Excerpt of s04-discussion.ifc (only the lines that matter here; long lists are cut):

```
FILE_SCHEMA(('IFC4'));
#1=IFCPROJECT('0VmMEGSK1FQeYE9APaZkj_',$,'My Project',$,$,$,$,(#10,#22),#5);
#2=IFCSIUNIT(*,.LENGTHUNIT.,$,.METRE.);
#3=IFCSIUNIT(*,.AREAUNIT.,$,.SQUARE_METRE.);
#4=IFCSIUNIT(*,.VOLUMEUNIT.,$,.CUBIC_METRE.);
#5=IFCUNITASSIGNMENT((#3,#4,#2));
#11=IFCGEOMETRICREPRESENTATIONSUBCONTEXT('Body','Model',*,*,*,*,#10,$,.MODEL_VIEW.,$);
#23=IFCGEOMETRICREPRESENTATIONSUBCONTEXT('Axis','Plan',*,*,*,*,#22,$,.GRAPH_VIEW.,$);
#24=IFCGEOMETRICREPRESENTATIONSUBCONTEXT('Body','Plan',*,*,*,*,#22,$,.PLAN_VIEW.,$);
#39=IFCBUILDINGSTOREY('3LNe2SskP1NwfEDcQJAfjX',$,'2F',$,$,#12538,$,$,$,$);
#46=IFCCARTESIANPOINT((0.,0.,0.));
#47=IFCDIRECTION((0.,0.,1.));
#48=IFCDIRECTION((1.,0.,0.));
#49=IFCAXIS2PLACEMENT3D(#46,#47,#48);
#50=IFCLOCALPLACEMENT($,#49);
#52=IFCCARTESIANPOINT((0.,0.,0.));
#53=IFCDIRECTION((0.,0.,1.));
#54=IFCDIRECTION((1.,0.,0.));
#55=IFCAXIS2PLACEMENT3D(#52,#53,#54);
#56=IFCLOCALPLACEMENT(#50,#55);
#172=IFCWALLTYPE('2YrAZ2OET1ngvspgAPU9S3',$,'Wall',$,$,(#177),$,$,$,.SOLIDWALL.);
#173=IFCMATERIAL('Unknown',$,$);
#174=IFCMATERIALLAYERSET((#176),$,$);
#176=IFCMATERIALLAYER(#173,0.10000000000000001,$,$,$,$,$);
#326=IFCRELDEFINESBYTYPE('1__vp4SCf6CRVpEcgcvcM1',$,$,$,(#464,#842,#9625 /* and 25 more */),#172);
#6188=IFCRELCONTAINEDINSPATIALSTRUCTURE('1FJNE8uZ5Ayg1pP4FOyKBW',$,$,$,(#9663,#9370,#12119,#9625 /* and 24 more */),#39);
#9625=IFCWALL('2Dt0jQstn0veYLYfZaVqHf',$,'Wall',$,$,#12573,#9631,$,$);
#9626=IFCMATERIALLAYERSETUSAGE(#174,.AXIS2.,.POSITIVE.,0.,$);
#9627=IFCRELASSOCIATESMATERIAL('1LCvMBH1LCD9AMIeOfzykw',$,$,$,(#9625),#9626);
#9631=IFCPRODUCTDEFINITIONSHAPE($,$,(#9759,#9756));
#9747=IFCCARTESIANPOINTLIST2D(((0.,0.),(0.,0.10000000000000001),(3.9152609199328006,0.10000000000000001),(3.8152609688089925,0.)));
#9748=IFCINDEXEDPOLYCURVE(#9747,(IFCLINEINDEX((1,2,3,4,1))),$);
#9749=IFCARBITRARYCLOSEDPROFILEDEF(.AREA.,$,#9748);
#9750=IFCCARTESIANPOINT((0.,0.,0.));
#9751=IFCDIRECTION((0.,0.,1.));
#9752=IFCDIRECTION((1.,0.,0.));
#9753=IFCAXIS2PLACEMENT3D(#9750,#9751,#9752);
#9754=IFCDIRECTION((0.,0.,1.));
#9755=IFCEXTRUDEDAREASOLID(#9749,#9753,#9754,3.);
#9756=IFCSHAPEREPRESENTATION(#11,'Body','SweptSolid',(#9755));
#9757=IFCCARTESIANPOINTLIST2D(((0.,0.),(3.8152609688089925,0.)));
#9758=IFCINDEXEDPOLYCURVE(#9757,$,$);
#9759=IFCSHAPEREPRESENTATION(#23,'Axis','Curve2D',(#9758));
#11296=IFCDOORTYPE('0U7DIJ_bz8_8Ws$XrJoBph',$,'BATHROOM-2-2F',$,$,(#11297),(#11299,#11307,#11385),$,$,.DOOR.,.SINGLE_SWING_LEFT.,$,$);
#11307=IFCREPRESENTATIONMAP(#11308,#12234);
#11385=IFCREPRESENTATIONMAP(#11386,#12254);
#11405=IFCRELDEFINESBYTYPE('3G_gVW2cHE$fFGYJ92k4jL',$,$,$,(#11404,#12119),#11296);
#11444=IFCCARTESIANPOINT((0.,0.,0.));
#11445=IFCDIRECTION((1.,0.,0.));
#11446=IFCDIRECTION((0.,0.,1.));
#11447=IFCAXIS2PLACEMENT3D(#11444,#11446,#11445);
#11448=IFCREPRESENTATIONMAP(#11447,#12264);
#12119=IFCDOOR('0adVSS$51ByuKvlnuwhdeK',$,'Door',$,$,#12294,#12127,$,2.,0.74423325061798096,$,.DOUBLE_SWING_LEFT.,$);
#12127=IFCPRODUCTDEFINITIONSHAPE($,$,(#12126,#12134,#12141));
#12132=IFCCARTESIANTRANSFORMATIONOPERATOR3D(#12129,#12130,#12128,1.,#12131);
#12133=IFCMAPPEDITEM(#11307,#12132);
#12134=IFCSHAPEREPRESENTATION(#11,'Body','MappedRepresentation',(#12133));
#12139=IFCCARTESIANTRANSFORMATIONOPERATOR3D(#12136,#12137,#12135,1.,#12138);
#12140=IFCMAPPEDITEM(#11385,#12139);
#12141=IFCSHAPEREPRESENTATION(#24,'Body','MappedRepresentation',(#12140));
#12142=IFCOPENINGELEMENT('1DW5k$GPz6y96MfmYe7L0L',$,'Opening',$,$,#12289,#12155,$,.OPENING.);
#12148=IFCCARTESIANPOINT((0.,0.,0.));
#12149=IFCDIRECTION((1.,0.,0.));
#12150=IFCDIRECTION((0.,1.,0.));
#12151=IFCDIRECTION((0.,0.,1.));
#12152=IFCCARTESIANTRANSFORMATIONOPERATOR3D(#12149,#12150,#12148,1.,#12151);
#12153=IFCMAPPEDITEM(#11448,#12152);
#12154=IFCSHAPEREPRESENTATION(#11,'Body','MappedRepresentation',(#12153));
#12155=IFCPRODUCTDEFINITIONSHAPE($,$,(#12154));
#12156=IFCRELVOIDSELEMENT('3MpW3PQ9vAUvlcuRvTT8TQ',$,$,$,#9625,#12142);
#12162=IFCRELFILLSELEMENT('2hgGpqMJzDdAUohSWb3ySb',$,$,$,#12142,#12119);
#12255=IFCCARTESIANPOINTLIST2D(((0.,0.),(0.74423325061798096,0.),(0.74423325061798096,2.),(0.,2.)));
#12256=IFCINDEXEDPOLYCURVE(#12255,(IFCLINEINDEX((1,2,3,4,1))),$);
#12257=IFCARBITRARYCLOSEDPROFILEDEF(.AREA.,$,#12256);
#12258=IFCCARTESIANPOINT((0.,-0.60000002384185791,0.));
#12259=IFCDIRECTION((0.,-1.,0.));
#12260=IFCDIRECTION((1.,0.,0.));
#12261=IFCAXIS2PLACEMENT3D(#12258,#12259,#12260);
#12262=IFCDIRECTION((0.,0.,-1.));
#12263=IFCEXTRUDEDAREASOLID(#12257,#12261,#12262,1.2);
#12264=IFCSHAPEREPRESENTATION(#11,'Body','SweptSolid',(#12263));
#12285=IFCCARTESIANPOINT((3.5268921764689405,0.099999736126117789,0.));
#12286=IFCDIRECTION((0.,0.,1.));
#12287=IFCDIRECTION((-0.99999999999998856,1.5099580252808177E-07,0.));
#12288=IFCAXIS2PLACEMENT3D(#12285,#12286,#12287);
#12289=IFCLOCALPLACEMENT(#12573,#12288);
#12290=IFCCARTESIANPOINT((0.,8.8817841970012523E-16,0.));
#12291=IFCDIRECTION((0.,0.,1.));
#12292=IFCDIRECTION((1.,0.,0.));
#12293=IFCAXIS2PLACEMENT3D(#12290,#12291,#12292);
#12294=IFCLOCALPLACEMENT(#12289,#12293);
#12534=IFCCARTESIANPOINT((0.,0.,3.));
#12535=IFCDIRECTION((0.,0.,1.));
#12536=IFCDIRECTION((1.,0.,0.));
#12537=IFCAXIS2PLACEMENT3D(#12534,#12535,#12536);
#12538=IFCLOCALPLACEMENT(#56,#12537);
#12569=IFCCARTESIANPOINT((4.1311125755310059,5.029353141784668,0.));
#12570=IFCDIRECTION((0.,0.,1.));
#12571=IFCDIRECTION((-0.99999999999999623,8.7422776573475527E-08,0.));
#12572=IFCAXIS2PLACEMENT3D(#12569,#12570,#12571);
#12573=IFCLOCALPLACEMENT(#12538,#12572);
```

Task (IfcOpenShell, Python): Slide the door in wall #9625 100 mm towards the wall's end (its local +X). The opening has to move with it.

```python
import ifcopenshell
import ifcopenshell.api.geometry
import ifcopenshell.util.placement

model = ifcopenshell.open("s04-discussion.ifc")

door = model.by_guid("0adVSS$51ByuKvlnuwhdeK")
opening = door.FillsVoids[0].RelatingOpeningElement
wall = opening.VoidsElements[0].RelatingBuildingElement

wall_matrix = ifcopenshell.util.placement.get_local_placement(wall.ObjectPlacement)
shift = wall_matrix[:3, 0] * 0.1
before = ifcopenshell.util.placement.get_local_placement(door.ObjectPlacement)[:3, 3].copy()

# The door is placed relative to its opening, so it follows when the opening moves.
matrix = ifcopenshell.util.placement.get_local_placement(opening.ObjectPlacement)
matrix[:3, 3] += shift
ifcopenshell.api.geometry.edit_object_placement(
    model, product=opening, matrix=matrix, is_si=False, should_transform_children=True
)

after = ifcopenshell.util.placement.get_local_placement(door.ObjectPlacement)[:3, 3]
print("door moved by", (after - before).round(3) + 0.0)

model.write("s04-discussion_edited.ifc")
```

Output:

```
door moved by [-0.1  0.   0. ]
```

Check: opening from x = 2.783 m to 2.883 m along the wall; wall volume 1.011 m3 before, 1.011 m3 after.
